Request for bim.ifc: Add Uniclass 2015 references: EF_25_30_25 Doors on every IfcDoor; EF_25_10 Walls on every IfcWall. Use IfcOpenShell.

First a look at what the model holds.

```python
import ifcopenshell

model = ifcopenshell.open("bim.ifc")
print(model.schema)
print("classifications:", [c.Name for c in model.by_type("IfcClassification")])
for ifc_class in ("IfcDoor", "IfcRoof", "IfcStair", "IfcWall", "IfcWindow"):
    print(ifc_class, len(model.by_type(ifc_class)))
```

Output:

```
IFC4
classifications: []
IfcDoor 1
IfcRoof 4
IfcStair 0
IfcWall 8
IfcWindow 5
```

```python
import ifcopenshell
import ifcopenshell.api.classification

model = ifcopenshell.open("bim.ifc")

system = ifcopenshell.api.classification.add_classification(model, classification="Uniclass 2015")

codes = {
    "IfcDoor": ("EF_25_30_25", "Doors"),
    "IfcWall": ("EF_25_10", "Walls"),
}
for ifc_class, (code, name) in codes.items():
    products = model.by_type(ifc_class)
    ifcopenshell.api.classification.add_reference(
        model, products=products, classification=system, identification=code, name=name
    )
    print(code, len(products))

model.write("bim-out.ifc")
```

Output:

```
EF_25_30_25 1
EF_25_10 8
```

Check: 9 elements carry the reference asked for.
